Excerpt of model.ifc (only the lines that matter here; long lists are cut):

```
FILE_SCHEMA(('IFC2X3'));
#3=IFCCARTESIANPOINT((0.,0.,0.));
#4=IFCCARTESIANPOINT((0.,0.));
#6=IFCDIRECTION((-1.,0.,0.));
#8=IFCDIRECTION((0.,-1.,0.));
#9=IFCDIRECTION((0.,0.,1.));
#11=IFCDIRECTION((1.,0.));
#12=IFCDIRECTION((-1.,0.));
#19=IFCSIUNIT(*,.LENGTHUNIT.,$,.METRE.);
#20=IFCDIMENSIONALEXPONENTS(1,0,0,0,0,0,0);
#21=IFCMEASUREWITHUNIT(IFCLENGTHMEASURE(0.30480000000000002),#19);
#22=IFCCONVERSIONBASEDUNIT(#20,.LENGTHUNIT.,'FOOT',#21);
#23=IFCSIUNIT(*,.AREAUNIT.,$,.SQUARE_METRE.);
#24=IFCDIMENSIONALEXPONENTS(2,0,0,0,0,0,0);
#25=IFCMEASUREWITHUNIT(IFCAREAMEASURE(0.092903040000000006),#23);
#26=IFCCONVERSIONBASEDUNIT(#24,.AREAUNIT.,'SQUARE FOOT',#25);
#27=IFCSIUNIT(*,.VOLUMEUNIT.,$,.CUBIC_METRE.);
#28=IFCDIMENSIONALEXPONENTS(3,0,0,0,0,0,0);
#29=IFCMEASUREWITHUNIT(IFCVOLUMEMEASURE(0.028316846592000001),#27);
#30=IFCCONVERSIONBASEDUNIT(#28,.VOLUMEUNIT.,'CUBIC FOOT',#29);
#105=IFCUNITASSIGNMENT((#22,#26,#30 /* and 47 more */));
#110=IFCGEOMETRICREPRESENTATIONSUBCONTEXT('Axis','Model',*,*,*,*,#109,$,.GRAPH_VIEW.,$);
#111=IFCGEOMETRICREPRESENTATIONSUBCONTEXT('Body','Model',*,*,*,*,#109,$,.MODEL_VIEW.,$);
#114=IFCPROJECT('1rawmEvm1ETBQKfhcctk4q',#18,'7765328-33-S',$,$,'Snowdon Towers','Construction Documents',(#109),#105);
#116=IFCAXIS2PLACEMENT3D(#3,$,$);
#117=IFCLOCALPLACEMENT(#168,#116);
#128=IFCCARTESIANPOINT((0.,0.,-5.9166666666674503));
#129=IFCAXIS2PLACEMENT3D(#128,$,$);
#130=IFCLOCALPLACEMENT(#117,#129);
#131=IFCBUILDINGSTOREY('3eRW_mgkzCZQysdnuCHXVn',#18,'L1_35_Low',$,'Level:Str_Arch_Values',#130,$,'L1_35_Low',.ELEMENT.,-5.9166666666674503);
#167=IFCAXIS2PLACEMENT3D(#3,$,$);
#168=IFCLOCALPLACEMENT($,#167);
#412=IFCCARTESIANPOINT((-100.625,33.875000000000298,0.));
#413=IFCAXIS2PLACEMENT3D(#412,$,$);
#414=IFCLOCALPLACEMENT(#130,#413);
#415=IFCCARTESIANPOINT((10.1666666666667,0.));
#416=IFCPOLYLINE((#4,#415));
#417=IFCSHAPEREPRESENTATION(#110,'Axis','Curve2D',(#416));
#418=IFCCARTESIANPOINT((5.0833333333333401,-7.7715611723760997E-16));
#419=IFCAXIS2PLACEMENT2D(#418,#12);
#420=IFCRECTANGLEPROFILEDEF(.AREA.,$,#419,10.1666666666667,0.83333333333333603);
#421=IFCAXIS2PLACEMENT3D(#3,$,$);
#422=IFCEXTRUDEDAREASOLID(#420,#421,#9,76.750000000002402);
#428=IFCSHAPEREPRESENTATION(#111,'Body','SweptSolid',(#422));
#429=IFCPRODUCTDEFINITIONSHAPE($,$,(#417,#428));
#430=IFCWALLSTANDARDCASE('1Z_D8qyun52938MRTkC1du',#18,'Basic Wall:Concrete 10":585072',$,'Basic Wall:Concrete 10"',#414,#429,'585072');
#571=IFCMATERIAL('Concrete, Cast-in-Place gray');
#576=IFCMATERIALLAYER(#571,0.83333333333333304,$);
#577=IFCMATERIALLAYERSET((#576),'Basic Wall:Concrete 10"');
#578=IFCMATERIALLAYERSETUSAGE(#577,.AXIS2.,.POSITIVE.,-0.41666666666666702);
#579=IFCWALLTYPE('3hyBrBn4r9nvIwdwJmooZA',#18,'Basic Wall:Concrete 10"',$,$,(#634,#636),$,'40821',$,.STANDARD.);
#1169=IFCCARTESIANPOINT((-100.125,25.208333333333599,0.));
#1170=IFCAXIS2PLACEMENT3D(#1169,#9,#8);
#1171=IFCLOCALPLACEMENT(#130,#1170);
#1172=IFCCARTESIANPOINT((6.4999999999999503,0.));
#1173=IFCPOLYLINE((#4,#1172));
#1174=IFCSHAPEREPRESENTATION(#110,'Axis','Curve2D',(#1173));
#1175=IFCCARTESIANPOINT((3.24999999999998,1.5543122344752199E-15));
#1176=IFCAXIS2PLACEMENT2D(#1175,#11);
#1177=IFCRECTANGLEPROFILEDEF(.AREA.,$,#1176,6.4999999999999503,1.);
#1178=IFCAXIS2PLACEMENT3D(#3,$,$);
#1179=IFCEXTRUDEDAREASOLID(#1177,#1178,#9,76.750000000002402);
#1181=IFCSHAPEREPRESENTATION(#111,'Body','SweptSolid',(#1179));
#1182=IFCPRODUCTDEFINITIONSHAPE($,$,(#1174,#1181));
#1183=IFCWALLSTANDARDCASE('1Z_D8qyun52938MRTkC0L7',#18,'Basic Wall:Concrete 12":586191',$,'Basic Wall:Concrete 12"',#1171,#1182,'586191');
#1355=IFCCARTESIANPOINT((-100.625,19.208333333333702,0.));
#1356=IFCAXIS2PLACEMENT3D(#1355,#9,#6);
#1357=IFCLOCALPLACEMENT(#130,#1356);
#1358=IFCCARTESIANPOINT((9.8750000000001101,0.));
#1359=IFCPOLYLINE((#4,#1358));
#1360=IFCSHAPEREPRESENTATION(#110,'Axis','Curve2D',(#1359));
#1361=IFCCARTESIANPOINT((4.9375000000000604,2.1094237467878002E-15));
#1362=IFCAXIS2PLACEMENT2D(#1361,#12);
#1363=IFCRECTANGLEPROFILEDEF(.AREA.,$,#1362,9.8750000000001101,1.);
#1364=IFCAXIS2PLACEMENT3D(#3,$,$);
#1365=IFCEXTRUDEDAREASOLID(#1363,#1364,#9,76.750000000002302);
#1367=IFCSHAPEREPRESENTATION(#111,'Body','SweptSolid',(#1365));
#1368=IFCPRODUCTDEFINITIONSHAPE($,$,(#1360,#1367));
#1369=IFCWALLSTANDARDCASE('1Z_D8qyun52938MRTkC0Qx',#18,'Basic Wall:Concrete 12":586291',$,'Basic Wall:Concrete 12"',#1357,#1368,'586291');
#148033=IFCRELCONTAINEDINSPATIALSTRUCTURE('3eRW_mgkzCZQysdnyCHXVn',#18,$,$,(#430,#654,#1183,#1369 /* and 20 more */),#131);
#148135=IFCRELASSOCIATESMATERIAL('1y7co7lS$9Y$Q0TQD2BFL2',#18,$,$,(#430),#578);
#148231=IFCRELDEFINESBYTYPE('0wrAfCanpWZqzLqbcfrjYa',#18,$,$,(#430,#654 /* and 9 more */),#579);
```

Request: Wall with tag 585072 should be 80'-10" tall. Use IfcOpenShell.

```python
import ifcopenshell
import ifcopenshell.geom
import ifcopenshell.util.representation
import ifcopenshell.util.shape
import ifcopenshell.util.unit

model = ifcopenshell.open("model.ifc")
unit_scale = ifcopenshell.util.unit.calculate_unit_scale(model)
settings = ifcopenshell.geom.settings()


def volume(element):
    """Net volume in cubic metres, openings subtracted."""
    shape = ifcopenshell.geom.create_shape(settings, element)
    return ifcopenshell.util.shape.get_volume(shape.geometry)


wall = model.by_guid("1Z_D8qyun52938MRTkC1du")
before = volume(wall)

body = ifcopenshell.util.representation.get_representation(wall, "Model", "Body")
solid = body.Items[0]
old_height = solid.Depth
solid.Depth = 970 * 0.0254 / unit_scale
after = volume(wall)

print(f"height {old_height:g} -> {solid.Depth:g}, volume {before:.3f} -> {after:.3f} m3")

model.write("model_rev.ifc")
```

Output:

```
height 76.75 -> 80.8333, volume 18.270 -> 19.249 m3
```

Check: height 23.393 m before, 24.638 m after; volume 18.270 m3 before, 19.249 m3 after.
